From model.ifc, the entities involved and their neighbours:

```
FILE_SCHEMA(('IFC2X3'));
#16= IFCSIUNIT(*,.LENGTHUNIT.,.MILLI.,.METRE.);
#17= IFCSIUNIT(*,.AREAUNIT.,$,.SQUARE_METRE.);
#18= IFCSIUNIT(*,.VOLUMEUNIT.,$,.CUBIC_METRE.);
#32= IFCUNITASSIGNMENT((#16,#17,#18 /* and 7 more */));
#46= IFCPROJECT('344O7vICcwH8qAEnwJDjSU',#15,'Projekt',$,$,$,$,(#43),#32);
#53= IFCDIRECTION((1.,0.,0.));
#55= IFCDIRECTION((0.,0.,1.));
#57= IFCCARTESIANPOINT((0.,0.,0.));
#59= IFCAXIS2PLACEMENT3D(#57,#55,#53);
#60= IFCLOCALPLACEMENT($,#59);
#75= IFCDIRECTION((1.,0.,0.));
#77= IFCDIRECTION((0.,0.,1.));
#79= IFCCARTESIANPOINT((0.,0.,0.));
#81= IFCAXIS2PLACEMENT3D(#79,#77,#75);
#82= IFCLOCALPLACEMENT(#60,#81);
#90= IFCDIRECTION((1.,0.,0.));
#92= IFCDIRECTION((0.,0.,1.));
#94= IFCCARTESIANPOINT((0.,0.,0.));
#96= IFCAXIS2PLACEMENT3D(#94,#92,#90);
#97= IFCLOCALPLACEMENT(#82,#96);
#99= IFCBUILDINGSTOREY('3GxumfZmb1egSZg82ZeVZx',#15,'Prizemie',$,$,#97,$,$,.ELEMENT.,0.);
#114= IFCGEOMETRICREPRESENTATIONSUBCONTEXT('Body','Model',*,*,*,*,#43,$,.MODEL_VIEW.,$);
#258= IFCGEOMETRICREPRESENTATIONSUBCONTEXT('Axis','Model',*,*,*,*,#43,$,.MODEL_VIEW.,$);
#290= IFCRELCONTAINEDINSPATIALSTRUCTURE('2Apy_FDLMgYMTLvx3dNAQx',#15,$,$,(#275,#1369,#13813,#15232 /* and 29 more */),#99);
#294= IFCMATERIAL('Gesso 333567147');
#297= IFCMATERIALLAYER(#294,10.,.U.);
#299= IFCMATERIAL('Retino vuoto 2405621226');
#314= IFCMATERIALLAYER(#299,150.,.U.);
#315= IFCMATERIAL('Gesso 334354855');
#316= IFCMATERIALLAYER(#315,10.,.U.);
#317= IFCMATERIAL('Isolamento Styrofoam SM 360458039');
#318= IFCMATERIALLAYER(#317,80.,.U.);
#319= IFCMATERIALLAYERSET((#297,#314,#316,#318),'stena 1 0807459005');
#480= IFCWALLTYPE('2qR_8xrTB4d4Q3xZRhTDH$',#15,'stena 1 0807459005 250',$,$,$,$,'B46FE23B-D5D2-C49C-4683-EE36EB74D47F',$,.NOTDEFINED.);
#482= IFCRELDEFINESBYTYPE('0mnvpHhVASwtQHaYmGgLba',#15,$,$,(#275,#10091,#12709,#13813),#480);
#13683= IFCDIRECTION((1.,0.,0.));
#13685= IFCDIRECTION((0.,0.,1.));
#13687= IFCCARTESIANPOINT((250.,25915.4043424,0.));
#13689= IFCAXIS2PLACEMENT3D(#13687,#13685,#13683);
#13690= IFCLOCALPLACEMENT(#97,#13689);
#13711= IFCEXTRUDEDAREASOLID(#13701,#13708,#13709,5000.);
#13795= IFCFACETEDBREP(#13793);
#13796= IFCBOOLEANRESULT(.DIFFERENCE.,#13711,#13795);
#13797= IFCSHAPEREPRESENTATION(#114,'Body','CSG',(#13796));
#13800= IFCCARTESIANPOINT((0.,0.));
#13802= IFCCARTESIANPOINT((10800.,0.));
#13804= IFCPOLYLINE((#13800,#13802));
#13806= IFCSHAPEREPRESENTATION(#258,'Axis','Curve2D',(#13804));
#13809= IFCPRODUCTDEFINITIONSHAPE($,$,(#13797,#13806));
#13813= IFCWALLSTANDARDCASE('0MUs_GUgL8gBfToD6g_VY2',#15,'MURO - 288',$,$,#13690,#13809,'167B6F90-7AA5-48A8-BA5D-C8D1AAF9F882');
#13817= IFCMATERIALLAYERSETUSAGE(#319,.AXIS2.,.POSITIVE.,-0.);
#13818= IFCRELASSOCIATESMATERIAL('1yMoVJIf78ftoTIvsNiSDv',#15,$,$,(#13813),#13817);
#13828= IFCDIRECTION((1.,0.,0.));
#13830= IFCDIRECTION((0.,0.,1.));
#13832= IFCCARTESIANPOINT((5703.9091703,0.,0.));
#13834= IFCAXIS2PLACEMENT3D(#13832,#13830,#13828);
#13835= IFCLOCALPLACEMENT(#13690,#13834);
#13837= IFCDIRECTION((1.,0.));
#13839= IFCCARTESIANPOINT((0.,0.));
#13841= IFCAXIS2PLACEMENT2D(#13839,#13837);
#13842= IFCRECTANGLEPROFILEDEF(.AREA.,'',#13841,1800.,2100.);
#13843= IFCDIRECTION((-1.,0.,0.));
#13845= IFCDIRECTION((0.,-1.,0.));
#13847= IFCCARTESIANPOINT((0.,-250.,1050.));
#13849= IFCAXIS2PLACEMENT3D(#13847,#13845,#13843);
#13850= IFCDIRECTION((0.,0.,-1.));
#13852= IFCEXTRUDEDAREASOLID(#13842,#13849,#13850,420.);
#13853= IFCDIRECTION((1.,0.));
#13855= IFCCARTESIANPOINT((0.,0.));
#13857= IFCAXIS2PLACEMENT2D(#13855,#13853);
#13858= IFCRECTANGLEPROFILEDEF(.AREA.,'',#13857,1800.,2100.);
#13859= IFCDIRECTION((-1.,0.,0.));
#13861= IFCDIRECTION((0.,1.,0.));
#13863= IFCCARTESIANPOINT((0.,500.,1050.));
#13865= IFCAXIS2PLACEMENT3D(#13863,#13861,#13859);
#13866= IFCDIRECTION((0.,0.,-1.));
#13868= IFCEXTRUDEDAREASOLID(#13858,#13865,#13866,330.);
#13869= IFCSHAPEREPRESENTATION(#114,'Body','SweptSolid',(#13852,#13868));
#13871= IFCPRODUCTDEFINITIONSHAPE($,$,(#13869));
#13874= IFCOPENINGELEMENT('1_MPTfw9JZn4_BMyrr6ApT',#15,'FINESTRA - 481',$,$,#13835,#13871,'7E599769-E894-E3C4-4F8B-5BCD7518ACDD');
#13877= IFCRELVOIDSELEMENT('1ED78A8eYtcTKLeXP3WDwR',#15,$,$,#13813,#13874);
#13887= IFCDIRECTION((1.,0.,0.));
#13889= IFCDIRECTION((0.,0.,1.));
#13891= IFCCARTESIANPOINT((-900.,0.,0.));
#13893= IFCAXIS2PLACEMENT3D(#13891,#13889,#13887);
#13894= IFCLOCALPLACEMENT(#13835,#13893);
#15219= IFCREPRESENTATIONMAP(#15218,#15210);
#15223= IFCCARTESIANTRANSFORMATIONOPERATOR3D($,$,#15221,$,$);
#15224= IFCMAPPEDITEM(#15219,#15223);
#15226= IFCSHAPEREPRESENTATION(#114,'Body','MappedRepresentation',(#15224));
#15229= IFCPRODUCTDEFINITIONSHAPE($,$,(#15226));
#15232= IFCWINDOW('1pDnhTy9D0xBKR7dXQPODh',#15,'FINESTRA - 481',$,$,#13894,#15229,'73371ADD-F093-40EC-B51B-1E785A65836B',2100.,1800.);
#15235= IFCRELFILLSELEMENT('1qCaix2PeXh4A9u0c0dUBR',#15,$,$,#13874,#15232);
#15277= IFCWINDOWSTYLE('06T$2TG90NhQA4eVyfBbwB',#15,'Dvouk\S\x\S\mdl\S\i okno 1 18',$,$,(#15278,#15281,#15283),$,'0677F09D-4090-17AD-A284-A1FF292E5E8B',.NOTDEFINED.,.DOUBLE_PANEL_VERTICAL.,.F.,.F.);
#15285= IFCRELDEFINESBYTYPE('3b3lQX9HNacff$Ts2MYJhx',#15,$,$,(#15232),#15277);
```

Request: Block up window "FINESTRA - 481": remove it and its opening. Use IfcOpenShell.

```python
import ifcopenshell
import ifcopenshell.api.feature
import ifcopenshell.api.root
import ifcopenshell.geom
import ifcopenshell.util.shape

model = ifcopenshell.open("model.ifc")
settings = ifcopenshell.geom.settings()


def volume(element):
    """Net volume in cubic metres, openings subtracted."""
    shape = ifcopenshell.geom.create_shape(settings, element)
    return ifcopenshell.util.shape.get_volume(shape.geometry)


window = model.by_guid("1pDnhTy9D0xBKR7dXQPODh")
opening = window.FillsVoids[0].RelatingOpeningElement
wall = opening.VoidsElements[0].RelatingBuildingElement
before = volume(wall)

ifcopenshell.api.root.remove_product(model, product=window)
ifcopenshell.api.feature.remove_feature(model, feature=opening)

after = volume(wall)

print(f"wall volume {before:.3f} -> {after:.3f} m3")

model.write("model_updated.ifc")
```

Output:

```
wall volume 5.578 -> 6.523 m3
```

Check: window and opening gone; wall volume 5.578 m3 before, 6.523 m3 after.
